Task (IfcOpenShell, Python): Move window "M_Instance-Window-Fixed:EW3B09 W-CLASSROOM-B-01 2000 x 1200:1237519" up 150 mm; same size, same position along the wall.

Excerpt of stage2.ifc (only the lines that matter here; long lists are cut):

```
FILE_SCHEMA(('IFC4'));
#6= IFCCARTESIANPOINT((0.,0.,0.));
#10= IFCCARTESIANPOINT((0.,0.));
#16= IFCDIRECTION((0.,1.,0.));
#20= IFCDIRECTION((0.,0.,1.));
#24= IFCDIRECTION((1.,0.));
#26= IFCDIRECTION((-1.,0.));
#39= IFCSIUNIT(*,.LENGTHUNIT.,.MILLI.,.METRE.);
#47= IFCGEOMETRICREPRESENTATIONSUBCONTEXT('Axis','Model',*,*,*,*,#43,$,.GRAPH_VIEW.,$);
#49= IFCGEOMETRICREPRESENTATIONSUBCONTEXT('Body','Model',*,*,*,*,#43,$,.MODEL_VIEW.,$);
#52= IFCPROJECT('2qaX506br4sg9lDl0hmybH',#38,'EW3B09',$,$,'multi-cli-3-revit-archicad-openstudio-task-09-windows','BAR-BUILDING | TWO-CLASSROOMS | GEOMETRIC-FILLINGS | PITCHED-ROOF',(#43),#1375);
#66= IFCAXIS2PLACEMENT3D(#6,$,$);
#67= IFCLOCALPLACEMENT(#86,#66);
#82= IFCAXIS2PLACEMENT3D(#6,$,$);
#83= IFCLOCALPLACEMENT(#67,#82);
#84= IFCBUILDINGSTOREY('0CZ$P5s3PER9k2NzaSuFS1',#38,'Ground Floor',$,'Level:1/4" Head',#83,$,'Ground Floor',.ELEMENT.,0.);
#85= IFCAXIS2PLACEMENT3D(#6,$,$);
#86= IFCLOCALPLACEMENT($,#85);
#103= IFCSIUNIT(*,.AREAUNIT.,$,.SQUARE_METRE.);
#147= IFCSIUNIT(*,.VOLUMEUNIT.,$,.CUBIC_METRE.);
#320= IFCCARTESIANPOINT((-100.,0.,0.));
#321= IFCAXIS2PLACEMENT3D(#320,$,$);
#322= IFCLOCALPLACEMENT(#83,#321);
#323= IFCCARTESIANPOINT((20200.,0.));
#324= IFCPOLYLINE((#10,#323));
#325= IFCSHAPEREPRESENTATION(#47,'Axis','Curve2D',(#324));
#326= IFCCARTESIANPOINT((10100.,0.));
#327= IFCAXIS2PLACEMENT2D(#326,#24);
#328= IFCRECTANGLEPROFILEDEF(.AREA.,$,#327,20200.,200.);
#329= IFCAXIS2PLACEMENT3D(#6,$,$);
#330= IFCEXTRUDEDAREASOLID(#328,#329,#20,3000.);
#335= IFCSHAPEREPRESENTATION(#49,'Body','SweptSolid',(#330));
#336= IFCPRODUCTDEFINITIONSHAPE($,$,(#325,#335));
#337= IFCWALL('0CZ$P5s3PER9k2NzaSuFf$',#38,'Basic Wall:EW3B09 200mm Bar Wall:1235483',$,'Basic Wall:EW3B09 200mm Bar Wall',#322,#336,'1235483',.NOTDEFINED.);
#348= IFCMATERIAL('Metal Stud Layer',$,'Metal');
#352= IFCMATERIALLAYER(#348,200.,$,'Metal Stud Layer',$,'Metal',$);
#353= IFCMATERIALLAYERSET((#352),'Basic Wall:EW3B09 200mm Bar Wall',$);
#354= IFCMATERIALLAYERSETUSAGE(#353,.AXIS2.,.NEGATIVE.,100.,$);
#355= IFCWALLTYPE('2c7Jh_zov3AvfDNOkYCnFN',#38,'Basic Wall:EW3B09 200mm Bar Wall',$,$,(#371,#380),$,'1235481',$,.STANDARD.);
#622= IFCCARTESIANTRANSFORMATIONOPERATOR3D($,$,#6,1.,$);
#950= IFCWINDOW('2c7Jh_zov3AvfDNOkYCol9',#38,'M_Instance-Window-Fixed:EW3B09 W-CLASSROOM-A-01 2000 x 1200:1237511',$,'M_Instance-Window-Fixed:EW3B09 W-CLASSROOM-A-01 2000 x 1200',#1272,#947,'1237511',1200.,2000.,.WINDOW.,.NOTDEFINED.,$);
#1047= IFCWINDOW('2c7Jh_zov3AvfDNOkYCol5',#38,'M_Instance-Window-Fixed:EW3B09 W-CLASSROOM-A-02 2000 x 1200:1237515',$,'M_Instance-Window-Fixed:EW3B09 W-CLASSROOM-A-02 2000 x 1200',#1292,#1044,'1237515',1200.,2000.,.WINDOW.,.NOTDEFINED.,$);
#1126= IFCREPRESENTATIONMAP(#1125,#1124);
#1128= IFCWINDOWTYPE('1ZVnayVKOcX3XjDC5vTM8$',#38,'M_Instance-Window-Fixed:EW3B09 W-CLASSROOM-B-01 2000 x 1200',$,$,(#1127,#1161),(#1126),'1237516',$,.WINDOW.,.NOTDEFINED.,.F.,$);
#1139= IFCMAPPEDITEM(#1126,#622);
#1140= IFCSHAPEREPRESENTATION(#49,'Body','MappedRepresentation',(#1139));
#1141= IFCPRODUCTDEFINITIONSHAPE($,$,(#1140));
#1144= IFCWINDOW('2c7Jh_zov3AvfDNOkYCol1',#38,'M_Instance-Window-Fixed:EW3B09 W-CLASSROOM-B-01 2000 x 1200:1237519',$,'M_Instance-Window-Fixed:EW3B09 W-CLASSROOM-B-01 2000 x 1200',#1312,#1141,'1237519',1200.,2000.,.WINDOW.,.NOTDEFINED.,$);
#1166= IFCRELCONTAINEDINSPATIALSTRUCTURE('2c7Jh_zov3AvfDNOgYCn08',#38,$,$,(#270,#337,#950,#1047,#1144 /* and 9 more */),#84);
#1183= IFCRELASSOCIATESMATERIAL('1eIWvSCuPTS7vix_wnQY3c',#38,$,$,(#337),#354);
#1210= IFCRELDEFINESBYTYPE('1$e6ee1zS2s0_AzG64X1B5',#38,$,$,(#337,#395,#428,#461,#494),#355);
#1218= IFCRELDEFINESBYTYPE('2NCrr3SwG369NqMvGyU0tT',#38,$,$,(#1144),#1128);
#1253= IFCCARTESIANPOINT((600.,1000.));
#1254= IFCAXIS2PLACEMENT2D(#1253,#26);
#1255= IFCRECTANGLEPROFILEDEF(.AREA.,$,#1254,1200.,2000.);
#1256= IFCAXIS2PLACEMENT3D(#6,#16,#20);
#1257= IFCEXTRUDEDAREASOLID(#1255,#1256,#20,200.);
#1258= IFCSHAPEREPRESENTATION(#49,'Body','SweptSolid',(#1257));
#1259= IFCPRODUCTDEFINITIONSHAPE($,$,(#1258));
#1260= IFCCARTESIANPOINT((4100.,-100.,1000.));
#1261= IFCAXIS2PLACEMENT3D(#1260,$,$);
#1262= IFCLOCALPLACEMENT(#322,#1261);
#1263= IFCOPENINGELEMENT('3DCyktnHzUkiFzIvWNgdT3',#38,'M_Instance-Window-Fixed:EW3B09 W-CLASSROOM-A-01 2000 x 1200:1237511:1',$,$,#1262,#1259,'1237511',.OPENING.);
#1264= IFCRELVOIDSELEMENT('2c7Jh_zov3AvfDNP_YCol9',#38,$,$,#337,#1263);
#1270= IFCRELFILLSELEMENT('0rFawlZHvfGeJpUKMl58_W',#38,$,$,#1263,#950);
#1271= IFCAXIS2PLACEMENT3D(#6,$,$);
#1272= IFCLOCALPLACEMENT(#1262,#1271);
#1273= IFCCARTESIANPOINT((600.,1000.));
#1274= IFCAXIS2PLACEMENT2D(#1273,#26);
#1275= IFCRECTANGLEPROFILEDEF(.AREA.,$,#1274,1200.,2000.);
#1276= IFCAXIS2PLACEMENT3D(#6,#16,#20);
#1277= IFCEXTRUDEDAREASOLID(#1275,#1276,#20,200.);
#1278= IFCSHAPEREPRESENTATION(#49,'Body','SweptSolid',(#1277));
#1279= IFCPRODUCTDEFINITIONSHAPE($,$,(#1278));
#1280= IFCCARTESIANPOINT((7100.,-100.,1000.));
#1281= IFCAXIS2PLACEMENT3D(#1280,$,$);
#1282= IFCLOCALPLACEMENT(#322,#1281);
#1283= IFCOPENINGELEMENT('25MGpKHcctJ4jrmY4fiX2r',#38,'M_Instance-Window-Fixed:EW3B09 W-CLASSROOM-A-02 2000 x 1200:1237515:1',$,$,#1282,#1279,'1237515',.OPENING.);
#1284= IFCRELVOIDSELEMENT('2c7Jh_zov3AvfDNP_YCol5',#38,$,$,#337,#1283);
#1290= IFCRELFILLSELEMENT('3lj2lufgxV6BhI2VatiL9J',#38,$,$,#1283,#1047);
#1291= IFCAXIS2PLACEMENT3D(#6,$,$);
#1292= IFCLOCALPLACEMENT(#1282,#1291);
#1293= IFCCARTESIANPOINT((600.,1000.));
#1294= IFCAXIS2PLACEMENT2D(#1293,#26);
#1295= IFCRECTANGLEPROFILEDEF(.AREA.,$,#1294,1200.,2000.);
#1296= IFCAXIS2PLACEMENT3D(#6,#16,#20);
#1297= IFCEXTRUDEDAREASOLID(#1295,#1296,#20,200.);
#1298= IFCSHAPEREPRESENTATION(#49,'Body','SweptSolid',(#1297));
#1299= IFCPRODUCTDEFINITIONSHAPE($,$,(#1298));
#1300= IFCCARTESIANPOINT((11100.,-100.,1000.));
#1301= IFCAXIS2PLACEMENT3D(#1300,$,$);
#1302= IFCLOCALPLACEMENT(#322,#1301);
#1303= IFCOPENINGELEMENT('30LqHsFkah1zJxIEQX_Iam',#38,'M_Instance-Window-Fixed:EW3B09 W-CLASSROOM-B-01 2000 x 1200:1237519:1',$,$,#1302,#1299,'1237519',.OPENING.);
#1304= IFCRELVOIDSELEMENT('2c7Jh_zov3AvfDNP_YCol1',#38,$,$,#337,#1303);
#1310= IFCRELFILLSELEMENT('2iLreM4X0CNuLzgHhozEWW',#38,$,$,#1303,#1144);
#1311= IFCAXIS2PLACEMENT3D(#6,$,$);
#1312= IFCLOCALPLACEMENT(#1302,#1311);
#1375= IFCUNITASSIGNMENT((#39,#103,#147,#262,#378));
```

```python
import numpy as np
import ifcopenshell
import ifcopenshell.api.geometry
import ifcopenshell.util.placement
import ifcopenshell.util.unit

model = ifcopenshell.open("stage2.ifc")
unit_scale = ifcopenshell.util.unit.calculate_unit_scale(model)

window = model.by_guid("2c7Jh_zov3AvfDNOkYCol1")
opening = window.FillsVoids[0].RelatingOpeningElement
dz = 150.0

shift = np.array([0.0, 0.0, dz])
# The window is placed relative to its opening, so it follows when the opening moves.
matrix = ifcopenshell.util.placement.get_local_placement(opening.ObjectPlacement)
matrix[:3, 3] += shift
ifcopenshell.api.geometry.edit_object_placement(
    model, product=opening, matrix=matrix, is_si=False, should_transform_children=True
)

print(f"moved by {dz * unit_scale:+.3f} m")

model.write("stage2-out.ifc")
```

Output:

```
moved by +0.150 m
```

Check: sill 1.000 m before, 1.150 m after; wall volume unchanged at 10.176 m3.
